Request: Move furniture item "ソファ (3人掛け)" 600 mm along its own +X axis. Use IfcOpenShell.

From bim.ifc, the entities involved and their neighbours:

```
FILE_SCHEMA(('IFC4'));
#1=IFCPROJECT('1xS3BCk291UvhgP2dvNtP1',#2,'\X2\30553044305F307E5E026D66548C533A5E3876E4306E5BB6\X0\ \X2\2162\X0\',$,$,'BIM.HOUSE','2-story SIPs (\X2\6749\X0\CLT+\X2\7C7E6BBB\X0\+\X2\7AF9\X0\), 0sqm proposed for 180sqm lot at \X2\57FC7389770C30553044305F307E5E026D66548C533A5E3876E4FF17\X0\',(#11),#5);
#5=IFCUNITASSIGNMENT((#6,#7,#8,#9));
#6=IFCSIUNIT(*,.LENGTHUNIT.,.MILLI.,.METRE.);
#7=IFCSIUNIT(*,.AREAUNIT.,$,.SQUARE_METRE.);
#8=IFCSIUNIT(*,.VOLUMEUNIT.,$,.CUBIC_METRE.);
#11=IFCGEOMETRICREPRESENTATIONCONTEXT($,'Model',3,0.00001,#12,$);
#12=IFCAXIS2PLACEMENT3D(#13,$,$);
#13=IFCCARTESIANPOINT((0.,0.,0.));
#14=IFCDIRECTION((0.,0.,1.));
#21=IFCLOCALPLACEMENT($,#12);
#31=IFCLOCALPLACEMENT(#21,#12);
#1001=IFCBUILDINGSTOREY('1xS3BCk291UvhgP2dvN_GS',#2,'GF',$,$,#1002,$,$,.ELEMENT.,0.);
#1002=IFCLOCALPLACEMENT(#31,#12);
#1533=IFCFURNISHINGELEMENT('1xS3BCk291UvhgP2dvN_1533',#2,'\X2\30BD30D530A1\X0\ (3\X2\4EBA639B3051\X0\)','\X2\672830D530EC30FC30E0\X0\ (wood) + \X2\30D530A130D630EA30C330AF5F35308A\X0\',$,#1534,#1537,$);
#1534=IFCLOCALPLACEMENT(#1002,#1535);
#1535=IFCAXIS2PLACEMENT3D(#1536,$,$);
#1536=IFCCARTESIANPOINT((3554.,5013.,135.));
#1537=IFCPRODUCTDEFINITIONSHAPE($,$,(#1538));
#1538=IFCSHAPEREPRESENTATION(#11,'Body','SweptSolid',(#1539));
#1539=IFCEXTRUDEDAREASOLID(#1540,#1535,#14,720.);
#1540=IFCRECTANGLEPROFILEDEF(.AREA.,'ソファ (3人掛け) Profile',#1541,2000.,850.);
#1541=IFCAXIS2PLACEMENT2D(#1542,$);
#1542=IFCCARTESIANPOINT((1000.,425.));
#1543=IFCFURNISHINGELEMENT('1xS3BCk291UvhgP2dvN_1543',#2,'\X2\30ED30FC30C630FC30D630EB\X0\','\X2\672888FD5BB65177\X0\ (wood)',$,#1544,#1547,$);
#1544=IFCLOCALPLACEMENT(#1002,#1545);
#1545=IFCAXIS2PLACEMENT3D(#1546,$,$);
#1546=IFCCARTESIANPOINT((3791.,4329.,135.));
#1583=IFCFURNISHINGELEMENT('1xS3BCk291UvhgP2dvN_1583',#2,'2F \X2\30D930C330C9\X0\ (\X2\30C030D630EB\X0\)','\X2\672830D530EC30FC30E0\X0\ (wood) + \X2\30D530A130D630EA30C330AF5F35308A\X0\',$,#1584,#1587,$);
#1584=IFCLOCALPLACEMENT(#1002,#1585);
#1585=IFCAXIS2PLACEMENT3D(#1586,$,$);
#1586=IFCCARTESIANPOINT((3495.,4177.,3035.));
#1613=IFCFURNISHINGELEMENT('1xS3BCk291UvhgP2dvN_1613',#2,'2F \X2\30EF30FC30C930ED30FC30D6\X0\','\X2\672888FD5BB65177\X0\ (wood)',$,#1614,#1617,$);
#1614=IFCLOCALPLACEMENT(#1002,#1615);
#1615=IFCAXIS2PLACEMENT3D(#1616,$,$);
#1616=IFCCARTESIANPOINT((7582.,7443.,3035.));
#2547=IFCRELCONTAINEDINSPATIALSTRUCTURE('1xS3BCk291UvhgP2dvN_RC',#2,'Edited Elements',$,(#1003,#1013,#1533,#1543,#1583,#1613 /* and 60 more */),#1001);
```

```python
import ifcopenshell
import ifcopenshell.api.geometry
import ifcopenshell.util.placement

model = ifcopenshell.open("bim.ifc")

item = model.by_id(1533)
matrix = ifcopenshell.util.placement.get_local_placement(item.ObjectPlacement)
matrix[:3, 3] += matrix[:3, 0] * 600.0
ifcopenshell.api.geometry.edit_object_placement(model, product=item, matrix=matrix, is_si=False)

print(ifcopenshell.util.placement.get_local_placement(item.ObjectPlacement).round(3) + 0.0)

model.write("bim_rev.ifc")
```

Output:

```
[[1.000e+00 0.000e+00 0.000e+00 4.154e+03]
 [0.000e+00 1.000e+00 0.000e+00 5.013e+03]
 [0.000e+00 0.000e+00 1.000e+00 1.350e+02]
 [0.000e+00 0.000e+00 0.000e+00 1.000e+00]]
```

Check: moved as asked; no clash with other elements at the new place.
